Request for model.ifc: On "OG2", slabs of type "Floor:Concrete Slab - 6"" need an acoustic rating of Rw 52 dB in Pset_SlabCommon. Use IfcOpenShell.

First a look at what the model holds.

```python
import ifcopenshell
import ifcopenshell.util.element

model = ifcopenshell.open("model.ifc")
print(model.schema)
storey = next(s for s in model.by_type("IfcBuildingStorey") if s.Name == "OG2")
slabs = [e for e in ifcopenshell.util.element.get_decomposition(storey) if e.is_a("IfcSlab")]
seen = {}
for e in slabs:
    element_type = ifcopenshell.util.element.get_type(e)
    key = (element_type.Name if element_type != e and element_type else None, ifcopenshell.util.element.get_pset(e, "Pset_SlabCommon", "AcousticRating"))
    seen[key] = seen.get(key, 0) + 1
for (name, value), count in sorted(seen.items(), key=str):
    print(count, "x", name, "|", value)
```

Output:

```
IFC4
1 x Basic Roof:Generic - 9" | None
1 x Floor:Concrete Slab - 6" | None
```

```python
import ifcopenshell
import ifcopenshell.api.pset
import ifcopenshell.util.element

model = ifcopenshell.open("model.ifc")

storey = next(s for s in model.by_type("IfcBuildingStorey") if s.Name == "OG2")
slabs = [e for e in ifcopenshell.util.element.get_decomposition(storey) if e.is_a("IfcSlab")]

count = 0
for e in slabs:
    element_type = ifcopenshell.util.element.get_type(e)
    if element_type in (None, e) or element_type.Name != 'Floor:Concrete Slab - 6"':
        continue
    # add_pset returns the element's existing set when there is one.
    pset = ifcopenshell.api.pset.add_pset(model, product=e, name="Pset_SlabCommon")
    ifcopenshell.api.pset.edit_pset(model, pset=pset, properties={"AcousticRating": "Rw 52 dB"})
    count += 1

print(count, "slabs updated")

model.write("model-out.ifc")
```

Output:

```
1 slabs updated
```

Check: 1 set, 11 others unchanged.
